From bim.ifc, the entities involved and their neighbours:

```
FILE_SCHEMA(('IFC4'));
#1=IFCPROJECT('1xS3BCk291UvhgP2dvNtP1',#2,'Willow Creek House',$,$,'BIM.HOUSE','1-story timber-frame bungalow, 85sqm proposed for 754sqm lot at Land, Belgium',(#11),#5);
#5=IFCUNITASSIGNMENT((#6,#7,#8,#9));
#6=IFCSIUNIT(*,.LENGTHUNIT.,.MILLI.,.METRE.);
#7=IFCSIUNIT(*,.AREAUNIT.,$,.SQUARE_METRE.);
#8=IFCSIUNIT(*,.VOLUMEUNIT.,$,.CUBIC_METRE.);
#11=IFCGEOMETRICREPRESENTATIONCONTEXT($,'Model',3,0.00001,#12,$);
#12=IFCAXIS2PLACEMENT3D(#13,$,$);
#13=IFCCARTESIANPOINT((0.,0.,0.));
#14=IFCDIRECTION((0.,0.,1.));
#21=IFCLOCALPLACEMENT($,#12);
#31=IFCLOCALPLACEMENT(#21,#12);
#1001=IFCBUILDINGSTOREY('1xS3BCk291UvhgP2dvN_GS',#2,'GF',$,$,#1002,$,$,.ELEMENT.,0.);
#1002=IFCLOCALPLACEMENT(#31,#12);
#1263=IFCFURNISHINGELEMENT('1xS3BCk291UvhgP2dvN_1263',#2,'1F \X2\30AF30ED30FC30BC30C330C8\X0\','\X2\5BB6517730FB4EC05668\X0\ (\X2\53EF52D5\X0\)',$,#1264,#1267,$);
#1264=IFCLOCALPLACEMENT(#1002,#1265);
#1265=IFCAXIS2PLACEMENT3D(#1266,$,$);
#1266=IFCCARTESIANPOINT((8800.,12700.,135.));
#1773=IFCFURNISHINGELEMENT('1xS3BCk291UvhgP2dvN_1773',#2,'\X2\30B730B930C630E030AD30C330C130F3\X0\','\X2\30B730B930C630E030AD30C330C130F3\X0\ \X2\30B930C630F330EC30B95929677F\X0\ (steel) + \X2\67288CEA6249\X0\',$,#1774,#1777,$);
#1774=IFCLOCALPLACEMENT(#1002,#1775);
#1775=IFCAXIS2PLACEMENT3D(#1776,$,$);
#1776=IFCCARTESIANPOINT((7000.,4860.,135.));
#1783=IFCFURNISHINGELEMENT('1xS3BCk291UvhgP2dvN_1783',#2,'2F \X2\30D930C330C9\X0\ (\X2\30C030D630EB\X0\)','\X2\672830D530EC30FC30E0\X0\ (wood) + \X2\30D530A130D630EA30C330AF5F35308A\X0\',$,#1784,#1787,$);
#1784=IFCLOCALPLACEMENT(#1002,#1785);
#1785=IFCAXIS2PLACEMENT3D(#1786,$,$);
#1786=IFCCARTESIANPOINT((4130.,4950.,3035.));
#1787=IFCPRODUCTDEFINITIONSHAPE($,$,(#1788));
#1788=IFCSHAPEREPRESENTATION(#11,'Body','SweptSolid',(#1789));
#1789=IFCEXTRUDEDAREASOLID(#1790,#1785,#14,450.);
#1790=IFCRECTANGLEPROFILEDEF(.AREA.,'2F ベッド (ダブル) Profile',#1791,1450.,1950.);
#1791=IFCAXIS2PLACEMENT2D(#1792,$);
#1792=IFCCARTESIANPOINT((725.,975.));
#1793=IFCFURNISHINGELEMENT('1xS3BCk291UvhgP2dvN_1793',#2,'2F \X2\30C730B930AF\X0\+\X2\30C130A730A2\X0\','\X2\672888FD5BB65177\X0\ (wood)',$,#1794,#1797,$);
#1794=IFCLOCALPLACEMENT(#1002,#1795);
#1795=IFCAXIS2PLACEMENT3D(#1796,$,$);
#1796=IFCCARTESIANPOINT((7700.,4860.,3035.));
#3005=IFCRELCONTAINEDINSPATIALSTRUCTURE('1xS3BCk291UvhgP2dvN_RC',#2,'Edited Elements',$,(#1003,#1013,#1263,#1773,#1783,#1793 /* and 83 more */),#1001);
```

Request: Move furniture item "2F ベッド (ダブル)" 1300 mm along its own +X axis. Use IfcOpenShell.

```python
import ifcopenshell
import ifcopenshell.api.geometry
import ifcopenshell.util.placement
import ifcopenshell.util.unit

model = ifcopenshell.open("bim.ifc")
unit_scale = ifcopenshell.util.unit.calculate_unit_scale(model)

item = model.by_guid("1xS3BCk291UvhgP2dvN_1783")
matrix = ifcopenshell.util.placement.get_local_placement(item.ObjectPlacement)
matrix[:3, 3] += matrix[:3, 0] * 1.3 / unit_scale
ifcopenshell.api.geometry.edit_object_placement(model, product=item, matrix=matrix, is_si=False)

print(ifcopenshell.util.placement.get_local_placement(item.ObjectPlacement).round(3) + 0.0)

model.write("bim_edited.ifc")
```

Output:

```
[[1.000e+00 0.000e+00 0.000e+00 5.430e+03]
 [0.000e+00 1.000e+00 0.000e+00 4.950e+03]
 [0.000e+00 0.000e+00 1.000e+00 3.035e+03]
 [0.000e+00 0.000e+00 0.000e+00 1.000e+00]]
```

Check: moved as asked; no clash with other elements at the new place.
